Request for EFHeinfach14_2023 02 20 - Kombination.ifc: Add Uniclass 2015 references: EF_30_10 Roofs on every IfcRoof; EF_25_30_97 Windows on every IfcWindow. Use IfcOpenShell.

First a look at what the model holds.

```python
import ifcopenshell

model = ifcopenshell.open("EFHeinfach14_2023 02 20 - Kombination.ifc")
print(model.schema)
print("classifications:", [c.Name for c in model.by_type("IfcClassification")])
for ifc_class in ("IfcDoor", "IfcRoof", "IfcStair", "IfcWall", "IfcWindow"):
    print(ifc_class, len(model.by_type(ifc_class)))
```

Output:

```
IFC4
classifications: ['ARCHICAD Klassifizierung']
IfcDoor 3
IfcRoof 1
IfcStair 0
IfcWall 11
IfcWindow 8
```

```python
import ifcopenshell
import ifcopenshell.api.classification

model = ifcopenshell.open("EFHeinfach14_2023 02 20 - Kombination.ifc")

system = ifcopenshell.api.classification.add_classification(model, classification="Uniclass 2015")

codes = {
    "IfcRoof": ("EF_30_10", "Roofs"),
    "IfcWindow": ("EF_25_30_97", "Windows"),
}
for ifc_class, (code, name) in codes.items():
    products = model.by_type(ifc_class)
    ifcopenshell.api.classification.add_reference(
        model, products=products, classification=system, identification=code, name=name
    )
    print(code, len(products))

model.write("EFHeinfach14_2023 02 20 - Kombination_edited.ifc")
```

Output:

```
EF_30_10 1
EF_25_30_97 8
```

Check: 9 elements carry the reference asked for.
